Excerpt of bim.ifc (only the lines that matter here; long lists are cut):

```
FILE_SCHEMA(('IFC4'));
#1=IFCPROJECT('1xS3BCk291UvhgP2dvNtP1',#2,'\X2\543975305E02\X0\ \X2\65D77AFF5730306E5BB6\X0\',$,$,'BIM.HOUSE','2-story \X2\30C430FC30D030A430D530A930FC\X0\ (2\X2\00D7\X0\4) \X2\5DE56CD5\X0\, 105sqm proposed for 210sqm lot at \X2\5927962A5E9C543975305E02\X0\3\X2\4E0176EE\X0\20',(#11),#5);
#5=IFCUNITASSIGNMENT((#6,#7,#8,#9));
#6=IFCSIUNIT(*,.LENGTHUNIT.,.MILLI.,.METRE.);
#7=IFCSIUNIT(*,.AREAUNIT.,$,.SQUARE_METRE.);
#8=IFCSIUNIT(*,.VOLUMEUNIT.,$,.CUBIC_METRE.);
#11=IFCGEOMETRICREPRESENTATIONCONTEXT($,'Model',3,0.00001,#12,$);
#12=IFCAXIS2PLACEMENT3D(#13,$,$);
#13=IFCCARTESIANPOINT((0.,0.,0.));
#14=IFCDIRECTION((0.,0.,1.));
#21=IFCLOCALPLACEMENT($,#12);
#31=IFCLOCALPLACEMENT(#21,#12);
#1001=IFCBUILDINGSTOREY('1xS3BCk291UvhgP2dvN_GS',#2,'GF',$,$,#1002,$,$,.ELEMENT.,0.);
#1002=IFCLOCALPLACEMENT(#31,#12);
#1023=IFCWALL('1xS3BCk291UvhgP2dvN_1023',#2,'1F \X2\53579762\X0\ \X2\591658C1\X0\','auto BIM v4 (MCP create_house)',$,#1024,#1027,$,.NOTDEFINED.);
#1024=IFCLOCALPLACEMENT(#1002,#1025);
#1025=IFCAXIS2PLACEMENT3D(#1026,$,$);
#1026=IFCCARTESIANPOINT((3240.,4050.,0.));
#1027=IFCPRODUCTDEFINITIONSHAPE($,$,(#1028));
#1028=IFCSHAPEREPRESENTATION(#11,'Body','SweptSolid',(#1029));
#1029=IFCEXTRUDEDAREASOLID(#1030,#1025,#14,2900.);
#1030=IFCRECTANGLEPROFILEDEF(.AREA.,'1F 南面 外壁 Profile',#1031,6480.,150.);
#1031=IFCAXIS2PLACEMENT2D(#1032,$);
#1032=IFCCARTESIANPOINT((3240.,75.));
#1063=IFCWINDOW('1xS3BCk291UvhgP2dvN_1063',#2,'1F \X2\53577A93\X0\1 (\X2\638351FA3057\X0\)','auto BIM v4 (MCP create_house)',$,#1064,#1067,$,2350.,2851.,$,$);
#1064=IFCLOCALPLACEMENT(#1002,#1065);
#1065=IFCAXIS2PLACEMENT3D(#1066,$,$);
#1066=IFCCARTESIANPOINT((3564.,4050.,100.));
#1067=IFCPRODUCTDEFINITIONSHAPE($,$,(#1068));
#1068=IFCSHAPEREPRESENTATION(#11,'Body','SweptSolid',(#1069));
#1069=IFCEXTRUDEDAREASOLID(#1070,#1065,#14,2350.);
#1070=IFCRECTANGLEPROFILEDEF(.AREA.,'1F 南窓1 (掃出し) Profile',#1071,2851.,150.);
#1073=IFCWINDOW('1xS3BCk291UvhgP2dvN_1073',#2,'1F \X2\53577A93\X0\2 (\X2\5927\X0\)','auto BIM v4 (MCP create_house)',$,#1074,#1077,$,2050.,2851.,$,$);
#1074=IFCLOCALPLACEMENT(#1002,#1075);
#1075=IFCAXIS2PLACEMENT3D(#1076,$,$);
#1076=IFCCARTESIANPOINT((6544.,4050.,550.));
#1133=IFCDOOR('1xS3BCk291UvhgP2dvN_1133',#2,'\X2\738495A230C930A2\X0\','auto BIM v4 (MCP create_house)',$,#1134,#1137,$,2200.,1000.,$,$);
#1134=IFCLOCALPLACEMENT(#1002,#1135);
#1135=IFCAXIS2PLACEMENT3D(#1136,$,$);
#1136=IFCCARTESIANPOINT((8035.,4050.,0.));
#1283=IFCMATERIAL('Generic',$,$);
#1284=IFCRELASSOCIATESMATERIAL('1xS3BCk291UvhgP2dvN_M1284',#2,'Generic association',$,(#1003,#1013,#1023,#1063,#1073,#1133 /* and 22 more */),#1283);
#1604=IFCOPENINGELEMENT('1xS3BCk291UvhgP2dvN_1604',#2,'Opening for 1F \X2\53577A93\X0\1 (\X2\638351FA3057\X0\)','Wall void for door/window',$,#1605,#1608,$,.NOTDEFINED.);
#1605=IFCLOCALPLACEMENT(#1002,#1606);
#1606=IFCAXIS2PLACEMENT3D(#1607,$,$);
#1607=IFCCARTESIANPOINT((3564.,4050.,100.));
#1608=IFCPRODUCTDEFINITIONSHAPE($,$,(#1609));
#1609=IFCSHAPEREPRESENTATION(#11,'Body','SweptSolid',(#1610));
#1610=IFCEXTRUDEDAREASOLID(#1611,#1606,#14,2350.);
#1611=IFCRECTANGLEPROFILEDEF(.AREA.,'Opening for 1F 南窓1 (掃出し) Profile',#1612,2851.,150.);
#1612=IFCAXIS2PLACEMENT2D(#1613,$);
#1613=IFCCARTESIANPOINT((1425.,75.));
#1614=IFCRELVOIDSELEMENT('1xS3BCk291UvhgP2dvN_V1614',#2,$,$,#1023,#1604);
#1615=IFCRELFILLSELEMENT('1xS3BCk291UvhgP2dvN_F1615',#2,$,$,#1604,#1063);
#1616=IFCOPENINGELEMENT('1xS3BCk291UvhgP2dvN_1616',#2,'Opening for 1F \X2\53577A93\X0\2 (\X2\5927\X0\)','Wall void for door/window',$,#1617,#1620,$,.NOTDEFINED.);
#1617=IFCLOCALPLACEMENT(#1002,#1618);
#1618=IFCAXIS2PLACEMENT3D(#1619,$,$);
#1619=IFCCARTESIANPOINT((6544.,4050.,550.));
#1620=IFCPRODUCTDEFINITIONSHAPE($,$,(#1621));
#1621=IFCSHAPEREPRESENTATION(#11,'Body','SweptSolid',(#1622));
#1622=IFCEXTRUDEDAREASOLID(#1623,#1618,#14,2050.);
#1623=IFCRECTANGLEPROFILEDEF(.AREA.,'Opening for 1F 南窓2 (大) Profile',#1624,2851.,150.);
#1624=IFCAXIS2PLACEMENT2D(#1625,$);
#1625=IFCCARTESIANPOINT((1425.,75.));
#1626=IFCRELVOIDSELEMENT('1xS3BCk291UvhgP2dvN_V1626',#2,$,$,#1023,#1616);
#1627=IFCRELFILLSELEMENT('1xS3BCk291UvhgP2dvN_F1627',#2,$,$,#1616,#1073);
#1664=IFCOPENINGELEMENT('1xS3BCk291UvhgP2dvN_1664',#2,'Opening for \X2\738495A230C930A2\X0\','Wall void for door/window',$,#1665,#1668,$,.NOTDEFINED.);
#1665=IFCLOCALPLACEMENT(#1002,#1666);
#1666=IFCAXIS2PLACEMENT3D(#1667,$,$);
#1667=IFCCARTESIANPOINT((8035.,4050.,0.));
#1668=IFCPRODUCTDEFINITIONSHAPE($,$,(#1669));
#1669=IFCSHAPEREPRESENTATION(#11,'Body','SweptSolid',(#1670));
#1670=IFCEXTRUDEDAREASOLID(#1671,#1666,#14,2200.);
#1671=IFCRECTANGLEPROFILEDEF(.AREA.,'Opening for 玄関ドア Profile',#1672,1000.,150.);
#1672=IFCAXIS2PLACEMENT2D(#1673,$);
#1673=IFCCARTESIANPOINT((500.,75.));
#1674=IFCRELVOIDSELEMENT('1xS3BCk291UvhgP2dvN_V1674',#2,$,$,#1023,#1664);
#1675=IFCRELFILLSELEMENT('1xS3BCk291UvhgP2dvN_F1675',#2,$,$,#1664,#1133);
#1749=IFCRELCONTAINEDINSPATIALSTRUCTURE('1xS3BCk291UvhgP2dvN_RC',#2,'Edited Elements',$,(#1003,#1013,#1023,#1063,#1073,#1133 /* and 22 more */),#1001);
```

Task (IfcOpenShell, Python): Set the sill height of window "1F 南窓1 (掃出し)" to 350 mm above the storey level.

```python
import numpy as np
import ifcopenshell
import ifcopenshell.api.geometry
import ifcopenshell.geom
import ifcopenshell.util.element
import ifcopenshell.util.placement
import ifcopenshell.util.shape
import ifcopenshell.util.unit

model = ifcopenshell.open("bim.ifc")
unit_scale = ifcopenshell.util.unit.calculate_unit_scale(model)

window = model.by_id(1063)
opening = window.FillsVoids[0].RelatingOpeningElement
storey = ifcopenshell.util.element.get_container(window, ifc_class="IfcBuildingStorey")
level = ifcopenshell.util.placement.get_local_placement(storey.ObjectPlacement)[2, 3]

# The opening's origin need not be at the sill, so measure its lowest point.
shape = ifcopenshell.geom.create_shape(ifcopenshell.geom.settings(), opening)
bottom = ifcopenshell.util.shape.get_shape_bottom_elevation(shape, shape.geometry) / unit_scale
dz = level + 0.35 / unit_scale - bottom

shift = np.array([0.0, 0.0, dz])
# The window is not placed relative to its opening, so move both.
for product in (opening, window):
    matrix = ifcopenshell.util.placement.get_local_placement(product.ObjectPlacement)
    matrix[:3, 3] += shift
    ifcopenshell.api.geometry.edit_object_placement(model, product=product, matrix=matrix, is_si=False)

print(f"moved by {dz * unit_scale:+.3f} m")

model.write("bim_v2.ifc")
```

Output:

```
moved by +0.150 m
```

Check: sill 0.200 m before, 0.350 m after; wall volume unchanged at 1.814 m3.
